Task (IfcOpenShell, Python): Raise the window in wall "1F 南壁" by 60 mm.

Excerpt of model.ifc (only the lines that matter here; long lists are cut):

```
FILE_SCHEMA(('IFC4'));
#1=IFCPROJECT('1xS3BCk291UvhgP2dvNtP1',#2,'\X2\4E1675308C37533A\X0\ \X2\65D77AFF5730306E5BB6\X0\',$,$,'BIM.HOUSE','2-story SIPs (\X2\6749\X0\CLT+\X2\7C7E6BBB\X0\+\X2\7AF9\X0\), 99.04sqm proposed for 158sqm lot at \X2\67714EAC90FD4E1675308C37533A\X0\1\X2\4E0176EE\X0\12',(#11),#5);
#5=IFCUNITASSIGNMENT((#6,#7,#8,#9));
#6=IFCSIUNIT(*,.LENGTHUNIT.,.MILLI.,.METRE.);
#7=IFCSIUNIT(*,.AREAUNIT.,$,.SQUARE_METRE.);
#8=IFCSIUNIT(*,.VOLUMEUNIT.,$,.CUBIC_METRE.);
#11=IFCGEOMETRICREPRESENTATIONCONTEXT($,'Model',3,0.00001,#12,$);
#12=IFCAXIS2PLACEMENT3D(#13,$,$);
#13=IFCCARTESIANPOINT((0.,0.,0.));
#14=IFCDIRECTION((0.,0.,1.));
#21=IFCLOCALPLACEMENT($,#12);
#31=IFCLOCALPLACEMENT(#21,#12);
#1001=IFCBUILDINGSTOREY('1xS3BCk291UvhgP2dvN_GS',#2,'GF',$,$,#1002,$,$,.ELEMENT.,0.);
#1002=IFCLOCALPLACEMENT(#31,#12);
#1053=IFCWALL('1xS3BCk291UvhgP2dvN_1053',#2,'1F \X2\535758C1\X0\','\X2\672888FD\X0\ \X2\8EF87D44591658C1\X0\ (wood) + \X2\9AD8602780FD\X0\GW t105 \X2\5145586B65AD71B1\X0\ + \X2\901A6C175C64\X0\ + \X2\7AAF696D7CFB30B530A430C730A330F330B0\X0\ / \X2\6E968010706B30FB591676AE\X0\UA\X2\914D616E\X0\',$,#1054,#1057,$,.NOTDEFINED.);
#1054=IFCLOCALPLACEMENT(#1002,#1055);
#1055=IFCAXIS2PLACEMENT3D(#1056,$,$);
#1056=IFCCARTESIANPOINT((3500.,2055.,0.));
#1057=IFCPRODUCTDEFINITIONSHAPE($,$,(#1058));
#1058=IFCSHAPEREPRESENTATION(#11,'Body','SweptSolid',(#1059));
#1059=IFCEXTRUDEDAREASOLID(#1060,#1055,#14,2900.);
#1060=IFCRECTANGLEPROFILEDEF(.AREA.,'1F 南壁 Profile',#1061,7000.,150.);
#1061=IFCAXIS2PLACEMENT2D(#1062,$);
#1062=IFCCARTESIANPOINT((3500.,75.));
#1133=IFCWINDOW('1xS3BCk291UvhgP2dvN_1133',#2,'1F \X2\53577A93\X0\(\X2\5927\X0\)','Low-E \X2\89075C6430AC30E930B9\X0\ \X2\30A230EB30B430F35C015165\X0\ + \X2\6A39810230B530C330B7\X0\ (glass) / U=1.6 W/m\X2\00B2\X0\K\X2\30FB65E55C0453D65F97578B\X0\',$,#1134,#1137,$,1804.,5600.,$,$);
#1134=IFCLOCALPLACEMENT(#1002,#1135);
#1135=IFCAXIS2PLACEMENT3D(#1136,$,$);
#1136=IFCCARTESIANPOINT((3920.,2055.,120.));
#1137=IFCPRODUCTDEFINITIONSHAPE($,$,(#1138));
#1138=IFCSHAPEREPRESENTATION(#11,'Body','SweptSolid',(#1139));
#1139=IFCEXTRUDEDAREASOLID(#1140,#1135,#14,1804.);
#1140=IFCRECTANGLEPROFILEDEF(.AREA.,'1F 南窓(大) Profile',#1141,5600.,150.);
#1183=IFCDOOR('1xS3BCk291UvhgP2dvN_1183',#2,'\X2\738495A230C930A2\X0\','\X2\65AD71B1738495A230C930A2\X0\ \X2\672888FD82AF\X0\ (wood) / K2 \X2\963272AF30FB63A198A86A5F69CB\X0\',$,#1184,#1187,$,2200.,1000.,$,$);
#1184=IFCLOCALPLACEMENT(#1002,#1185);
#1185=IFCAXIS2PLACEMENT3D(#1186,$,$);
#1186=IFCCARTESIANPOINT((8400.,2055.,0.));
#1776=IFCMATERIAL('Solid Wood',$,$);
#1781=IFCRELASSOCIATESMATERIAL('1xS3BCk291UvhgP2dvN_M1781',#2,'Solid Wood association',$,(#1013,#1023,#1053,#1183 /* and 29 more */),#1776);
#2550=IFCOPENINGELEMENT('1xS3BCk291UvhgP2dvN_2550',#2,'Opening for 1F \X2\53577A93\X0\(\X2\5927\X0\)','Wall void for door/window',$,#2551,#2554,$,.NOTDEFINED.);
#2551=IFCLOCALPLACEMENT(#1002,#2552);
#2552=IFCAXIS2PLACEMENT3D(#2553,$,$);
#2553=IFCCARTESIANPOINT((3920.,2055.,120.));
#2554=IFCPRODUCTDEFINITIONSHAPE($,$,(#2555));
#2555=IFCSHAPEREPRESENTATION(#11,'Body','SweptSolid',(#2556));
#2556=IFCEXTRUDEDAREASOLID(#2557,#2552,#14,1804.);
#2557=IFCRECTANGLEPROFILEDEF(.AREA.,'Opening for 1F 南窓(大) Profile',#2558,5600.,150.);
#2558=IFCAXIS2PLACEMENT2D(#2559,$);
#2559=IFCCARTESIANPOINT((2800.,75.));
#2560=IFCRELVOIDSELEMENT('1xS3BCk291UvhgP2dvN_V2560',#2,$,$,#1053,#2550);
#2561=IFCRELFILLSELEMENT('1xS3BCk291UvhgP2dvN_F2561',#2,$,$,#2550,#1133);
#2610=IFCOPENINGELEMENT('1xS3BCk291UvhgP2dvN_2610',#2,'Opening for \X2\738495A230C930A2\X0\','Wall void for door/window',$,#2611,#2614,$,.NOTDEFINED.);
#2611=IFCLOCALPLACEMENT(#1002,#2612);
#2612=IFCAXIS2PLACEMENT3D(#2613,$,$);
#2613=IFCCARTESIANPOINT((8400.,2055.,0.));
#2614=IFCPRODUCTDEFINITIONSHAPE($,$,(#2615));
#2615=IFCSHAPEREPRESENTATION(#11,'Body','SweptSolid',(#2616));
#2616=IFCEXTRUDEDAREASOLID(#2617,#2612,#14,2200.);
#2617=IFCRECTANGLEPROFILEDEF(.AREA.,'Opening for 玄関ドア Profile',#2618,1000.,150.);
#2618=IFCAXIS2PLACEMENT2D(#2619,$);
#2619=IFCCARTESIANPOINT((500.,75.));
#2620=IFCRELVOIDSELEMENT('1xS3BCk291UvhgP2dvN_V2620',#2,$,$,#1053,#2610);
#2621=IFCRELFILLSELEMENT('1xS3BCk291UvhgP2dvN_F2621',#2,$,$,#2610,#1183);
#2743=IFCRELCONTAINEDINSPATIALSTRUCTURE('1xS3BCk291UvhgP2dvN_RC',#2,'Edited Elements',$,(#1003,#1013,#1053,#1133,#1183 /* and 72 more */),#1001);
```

```python
import numpy as np
import ifcopenshell
import ifcopenshell.api.geometry
import ifcopenshell.util.placement
import ifcopenshell.util.unit

model = ifcopenshell.open("model.ifc")
unit_scale = ifcopenshell.util.unit.calculate_unit_scale(model)

window = model.by_id(1133)
opening = window.FillsVoids[0].RelatingOpeningElement
dz = 0.06 / unit_scale

shift = np.array([0.0, 0.0, dz])
# The window is not placed relative to its opening, so move both.
for product in (opening, window):
    matrix = ifcopenshell.util.placement.get_local_placement(product.ObjectPlacement)
    matrix[:3, 3] += shift
    ifcopenshell.api.geometry.edit_object_placement(model, product=product, matrix=matrix, is_si=False)

print(f"moved by {dz * unit_scale:+.3f} m")

model.write("model_edited.ifc")
```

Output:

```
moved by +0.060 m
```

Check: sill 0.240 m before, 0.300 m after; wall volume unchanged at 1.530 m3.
